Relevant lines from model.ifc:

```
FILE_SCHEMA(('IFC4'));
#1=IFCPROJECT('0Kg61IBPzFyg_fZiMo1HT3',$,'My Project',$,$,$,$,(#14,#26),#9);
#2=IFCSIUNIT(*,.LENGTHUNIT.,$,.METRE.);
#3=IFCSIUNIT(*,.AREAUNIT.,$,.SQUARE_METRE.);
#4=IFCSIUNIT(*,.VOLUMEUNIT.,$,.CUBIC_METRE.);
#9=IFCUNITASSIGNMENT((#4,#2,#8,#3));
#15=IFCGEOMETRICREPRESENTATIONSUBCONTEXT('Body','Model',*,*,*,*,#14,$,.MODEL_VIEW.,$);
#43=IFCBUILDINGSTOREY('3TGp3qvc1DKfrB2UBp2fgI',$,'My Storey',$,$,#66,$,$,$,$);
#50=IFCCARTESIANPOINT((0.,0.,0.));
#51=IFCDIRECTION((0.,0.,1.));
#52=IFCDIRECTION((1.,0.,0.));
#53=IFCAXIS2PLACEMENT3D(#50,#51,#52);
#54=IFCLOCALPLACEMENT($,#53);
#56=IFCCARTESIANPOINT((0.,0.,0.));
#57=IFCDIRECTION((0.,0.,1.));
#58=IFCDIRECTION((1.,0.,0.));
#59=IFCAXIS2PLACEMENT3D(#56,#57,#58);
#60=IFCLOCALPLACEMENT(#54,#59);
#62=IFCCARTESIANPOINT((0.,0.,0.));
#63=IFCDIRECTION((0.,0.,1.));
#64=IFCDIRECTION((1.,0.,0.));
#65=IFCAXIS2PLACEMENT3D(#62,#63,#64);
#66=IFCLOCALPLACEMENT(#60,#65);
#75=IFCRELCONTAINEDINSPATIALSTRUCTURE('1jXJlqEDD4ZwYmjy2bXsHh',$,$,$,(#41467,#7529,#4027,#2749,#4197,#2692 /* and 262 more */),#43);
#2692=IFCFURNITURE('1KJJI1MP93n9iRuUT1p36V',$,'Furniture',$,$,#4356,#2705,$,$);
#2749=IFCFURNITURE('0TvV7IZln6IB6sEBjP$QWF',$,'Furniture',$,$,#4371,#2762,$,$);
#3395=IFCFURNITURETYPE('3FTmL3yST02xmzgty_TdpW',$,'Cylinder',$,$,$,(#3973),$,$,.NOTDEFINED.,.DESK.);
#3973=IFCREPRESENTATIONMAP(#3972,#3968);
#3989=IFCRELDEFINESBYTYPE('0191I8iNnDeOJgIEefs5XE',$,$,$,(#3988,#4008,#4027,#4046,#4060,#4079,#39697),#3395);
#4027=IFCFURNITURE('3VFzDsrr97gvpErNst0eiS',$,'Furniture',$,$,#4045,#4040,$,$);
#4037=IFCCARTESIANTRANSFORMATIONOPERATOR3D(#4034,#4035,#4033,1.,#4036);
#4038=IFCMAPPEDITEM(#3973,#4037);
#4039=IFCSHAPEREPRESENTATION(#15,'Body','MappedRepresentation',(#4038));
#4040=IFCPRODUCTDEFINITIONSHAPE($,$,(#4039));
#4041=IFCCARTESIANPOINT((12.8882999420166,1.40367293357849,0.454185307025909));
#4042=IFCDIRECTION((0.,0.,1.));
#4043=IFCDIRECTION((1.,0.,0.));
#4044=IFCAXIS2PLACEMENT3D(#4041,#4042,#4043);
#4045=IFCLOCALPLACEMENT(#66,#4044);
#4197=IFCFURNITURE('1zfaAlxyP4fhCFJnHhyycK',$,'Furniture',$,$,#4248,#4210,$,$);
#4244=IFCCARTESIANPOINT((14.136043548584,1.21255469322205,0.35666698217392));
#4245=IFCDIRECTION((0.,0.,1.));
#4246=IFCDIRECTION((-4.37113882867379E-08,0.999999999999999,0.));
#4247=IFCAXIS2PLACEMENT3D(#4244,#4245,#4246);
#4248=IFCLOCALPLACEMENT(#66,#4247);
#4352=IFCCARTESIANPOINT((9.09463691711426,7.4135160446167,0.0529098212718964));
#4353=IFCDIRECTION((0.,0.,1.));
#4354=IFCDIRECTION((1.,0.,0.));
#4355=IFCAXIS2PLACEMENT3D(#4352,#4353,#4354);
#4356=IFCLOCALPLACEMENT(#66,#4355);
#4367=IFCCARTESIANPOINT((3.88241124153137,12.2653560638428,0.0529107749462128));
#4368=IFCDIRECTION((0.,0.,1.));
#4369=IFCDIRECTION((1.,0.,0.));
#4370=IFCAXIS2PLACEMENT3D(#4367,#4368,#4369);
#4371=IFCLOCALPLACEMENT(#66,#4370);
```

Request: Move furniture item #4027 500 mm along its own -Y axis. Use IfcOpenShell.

```python
import ifcopenshell
import ifcopenshell.api.geometry
import ifcopenshell.util.placement

model = ifcopenshell.open("model.ifc")

item = model.by_id(4027)
matrix = ifcopenshell.util.placement.get_local_placement(item.ObjectPlacement)
matrix[:3, 3] -= matrix[:3, 1] * 0.5
ifcopenshell.api.geometry.edit_object_placement(model, product=item, matrix=matrix, is_si=False)

print(ifcopenshell.util.placement.get_local_placement(item.ObjectPlacement).round(3) + 0.0)

model.write("model_updated.ifc")
```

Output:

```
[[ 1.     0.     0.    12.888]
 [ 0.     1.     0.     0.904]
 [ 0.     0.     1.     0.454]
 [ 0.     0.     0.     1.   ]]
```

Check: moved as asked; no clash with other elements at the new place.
